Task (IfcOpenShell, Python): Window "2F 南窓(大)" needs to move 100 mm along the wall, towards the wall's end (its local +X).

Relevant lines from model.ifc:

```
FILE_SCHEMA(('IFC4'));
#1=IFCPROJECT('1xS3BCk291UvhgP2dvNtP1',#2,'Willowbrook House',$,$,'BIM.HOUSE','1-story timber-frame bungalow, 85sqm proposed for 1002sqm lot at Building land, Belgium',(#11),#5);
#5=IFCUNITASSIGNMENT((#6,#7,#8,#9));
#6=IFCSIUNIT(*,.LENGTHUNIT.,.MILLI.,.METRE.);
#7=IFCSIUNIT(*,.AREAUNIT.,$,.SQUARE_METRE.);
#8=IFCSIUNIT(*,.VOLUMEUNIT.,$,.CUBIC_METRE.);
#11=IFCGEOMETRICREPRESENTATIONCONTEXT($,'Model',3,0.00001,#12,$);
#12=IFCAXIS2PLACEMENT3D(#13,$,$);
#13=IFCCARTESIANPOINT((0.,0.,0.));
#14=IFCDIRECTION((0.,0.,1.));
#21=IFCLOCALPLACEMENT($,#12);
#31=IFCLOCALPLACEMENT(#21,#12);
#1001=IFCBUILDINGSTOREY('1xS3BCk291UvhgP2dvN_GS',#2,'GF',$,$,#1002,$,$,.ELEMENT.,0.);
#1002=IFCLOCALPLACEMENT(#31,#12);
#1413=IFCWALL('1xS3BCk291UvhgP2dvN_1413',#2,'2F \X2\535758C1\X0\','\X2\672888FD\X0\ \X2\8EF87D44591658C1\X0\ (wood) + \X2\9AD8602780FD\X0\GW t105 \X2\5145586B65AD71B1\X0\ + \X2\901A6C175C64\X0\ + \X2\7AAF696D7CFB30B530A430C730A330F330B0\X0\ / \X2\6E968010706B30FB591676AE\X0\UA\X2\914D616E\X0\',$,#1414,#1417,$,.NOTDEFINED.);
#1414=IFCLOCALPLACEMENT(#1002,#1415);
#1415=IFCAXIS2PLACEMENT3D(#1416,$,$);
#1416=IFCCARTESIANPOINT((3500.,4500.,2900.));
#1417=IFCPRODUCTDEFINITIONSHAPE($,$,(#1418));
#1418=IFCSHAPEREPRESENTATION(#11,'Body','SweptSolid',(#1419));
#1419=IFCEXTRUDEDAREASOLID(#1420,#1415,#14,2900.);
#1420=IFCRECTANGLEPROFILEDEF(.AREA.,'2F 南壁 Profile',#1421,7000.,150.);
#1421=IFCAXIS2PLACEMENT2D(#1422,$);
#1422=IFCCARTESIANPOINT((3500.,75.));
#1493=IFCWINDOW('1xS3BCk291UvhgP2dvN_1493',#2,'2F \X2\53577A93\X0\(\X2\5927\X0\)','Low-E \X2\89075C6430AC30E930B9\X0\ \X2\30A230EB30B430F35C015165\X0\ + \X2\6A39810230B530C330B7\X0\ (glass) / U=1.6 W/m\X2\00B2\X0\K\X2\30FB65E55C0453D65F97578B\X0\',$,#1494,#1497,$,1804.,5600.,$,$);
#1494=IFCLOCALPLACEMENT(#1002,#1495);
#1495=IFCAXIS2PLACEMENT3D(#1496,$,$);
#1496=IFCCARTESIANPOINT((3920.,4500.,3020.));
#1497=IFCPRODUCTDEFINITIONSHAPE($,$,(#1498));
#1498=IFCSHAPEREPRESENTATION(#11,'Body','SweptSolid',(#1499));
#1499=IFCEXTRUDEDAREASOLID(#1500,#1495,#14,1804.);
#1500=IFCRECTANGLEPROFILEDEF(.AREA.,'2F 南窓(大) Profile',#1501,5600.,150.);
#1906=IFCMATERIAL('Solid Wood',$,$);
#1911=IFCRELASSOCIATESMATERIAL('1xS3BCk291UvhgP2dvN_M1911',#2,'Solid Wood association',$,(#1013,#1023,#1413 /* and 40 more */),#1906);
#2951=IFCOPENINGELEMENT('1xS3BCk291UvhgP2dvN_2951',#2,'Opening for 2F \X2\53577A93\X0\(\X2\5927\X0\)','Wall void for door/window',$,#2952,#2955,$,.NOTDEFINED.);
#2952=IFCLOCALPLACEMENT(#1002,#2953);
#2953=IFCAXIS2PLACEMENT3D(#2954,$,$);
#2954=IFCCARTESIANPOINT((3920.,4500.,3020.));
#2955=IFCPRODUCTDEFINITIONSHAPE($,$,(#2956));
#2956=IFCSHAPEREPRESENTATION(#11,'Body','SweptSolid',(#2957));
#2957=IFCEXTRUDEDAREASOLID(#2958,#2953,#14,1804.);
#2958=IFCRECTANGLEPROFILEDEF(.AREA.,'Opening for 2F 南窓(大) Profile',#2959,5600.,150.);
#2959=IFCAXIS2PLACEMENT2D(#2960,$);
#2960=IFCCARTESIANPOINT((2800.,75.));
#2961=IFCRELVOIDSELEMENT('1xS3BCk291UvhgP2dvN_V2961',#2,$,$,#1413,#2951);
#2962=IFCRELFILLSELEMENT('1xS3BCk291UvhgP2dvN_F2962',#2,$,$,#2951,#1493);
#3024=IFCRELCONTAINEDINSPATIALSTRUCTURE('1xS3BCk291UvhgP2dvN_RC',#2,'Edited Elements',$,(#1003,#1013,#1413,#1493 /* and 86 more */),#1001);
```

```python
import ifcopenshell
import ifcopenshell.api.geometry
import ifcopenshell.util.placement

model = ifcopenshell.open("model.ifc")

window = model.by_id(1493)
opening = window.FillsVoids[0].RelatingOpeningElement
wall = opening.VoidsElements[0].RelatingBuildingElement

wall_matrix = ifcopenshell.util.placement.get_local_placement(wall.ObjectPlacement)
shift = wall_matrix[:3, 0] * 100.0
before = ifcopenshell.util.placement.get_local_placement(window.ObjectPlacement)[:3, 3].copy()

# The window is not placed relative to its opening, so move both.
for product in (opening, window):
    matrix = ifcopenshell.util.placement.get_local_placement(product.ObjectPlacement)
    matrix[:3, 3] += shift
    ifcopenshell.api.geometry.edit_object_placement(model, product=product, matrix=matrix, is_si=False)

after = ifcopenshell.util.placement.get_local_placement(window.ObjectPlacement)[:3, 3]
print("window moved by", (after - before).round(3) + 0.0)

model.write("model_updated.ifc")
```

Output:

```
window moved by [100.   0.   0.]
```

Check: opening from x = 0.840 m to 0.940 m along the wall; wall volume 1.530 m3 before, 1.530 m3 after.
